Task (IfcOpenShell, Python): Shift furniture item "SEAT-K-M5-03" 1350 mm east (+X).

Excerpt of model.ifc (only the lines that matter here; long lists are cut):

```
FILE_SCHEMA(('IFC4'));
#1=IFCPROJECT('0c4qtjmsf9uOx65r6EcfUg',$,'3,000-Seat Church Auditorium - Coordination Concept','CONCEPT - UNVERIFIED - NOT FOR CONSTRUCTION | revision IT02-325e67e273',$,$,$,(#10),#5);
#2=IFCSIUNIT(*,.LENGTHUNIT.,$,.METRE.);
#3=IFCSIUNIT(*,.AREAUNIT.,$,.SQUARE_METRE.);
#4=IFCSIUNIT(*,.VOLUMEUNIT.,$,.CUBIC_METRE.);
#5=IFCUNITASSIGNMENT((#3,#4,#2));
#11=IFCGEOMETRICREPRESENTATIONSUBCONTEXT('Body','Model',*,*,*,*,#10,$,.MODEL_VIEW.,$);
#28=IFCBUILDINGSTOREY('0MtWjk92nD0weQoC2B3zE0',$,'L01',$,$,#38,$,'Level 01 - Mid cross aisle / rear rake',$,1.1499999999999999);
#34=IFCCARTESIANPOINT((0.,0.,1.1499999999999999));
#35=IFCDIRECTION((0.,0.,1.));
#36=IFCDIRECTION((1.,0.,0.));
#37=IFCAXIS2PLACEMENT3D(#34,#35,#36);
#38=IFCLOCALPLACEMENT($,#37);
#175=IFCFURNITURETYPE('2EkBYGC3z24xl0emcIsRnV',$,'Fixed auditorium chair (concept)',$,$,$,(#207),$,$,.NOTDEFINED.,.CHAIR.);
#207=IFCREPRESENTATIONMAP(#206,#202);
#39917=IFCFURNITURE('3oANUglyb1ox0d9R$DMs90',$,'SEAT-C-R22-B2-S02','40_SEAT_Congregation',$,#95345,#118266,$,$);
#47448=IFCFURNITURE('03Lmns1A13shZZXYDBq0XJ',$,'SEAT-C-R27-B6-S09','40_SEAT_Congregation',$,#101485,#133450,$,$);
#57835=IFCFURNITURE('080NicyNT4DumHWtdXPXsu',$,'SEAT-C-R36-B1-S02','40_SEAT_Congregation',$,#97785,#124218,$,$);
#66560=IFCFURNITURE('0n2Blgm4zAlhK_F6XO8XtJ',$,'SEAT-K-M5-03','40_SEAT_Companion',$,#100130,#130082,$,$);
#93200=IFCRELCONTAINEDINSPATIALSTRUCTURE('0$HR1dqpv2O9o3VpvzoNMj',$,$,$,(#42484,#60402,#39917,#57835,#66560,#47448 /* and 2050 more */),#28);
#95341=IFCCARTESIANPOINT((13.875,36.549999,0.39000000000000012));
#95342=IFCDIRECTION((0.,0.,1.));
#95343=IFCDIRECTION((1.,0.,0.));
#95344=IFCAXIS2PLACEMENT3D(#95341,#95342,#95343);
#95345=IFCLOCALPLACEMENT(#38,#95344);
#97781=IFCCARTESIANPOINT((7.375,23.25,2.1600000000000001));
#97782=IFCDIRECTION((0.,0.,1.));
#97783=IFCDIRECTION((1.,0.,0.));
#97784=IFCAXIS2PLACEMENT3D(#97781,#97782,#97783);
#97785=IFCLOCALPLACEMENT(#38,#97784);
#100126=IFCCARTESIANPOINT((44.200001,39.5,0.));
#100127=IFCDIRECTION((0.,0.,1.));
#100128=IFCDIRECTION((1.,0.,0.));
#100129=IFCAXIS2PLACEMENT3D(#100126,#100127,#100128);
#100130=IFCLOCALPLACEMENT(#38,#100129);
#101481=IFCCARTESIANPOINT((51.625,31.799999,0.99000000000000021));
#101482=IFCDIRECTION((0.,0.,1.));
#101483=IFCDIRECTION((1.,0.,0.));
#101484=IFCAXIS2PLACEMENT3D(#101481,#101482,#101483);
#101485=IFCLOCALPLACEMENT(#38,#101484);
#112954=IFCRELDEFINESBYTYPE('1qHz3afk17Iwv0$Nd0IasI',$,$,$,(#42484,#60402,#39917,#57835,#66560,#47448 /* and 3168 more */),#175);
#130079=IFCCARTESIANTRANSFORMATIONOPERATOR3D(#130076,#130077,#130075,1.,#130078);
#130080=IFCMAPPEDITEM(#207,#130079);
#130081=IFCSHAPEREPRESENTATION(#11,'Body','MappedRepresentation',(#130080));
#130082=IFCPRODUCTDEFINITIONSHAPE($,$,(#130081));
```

```python
import ifcopenshell
import ifcopenshell.api.geometry
import ifcopenshell.util.placement

model = ifcopenshell.open("model.ifc")

item = model.by_id(66560)
matrix = ifcopenshell.util.placement.get_local_placement(item.ObjectPlacement)
matrix[0, 3] += 1.35
ifcopenshell.api.geometry.edit_object_placement(model, product=item, matrix=matrix, is_si=False)

print(ifcopenshell.util.placement.get_local_placement(item.ObjectPlacement).round(3) + 0.0)

model.write("model_updated.ifc")
```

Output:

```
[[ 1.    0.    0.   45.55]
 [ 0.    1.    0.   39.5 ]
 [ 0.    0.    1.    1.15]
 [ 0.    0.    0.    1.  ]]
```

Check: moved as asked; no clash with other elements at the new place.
